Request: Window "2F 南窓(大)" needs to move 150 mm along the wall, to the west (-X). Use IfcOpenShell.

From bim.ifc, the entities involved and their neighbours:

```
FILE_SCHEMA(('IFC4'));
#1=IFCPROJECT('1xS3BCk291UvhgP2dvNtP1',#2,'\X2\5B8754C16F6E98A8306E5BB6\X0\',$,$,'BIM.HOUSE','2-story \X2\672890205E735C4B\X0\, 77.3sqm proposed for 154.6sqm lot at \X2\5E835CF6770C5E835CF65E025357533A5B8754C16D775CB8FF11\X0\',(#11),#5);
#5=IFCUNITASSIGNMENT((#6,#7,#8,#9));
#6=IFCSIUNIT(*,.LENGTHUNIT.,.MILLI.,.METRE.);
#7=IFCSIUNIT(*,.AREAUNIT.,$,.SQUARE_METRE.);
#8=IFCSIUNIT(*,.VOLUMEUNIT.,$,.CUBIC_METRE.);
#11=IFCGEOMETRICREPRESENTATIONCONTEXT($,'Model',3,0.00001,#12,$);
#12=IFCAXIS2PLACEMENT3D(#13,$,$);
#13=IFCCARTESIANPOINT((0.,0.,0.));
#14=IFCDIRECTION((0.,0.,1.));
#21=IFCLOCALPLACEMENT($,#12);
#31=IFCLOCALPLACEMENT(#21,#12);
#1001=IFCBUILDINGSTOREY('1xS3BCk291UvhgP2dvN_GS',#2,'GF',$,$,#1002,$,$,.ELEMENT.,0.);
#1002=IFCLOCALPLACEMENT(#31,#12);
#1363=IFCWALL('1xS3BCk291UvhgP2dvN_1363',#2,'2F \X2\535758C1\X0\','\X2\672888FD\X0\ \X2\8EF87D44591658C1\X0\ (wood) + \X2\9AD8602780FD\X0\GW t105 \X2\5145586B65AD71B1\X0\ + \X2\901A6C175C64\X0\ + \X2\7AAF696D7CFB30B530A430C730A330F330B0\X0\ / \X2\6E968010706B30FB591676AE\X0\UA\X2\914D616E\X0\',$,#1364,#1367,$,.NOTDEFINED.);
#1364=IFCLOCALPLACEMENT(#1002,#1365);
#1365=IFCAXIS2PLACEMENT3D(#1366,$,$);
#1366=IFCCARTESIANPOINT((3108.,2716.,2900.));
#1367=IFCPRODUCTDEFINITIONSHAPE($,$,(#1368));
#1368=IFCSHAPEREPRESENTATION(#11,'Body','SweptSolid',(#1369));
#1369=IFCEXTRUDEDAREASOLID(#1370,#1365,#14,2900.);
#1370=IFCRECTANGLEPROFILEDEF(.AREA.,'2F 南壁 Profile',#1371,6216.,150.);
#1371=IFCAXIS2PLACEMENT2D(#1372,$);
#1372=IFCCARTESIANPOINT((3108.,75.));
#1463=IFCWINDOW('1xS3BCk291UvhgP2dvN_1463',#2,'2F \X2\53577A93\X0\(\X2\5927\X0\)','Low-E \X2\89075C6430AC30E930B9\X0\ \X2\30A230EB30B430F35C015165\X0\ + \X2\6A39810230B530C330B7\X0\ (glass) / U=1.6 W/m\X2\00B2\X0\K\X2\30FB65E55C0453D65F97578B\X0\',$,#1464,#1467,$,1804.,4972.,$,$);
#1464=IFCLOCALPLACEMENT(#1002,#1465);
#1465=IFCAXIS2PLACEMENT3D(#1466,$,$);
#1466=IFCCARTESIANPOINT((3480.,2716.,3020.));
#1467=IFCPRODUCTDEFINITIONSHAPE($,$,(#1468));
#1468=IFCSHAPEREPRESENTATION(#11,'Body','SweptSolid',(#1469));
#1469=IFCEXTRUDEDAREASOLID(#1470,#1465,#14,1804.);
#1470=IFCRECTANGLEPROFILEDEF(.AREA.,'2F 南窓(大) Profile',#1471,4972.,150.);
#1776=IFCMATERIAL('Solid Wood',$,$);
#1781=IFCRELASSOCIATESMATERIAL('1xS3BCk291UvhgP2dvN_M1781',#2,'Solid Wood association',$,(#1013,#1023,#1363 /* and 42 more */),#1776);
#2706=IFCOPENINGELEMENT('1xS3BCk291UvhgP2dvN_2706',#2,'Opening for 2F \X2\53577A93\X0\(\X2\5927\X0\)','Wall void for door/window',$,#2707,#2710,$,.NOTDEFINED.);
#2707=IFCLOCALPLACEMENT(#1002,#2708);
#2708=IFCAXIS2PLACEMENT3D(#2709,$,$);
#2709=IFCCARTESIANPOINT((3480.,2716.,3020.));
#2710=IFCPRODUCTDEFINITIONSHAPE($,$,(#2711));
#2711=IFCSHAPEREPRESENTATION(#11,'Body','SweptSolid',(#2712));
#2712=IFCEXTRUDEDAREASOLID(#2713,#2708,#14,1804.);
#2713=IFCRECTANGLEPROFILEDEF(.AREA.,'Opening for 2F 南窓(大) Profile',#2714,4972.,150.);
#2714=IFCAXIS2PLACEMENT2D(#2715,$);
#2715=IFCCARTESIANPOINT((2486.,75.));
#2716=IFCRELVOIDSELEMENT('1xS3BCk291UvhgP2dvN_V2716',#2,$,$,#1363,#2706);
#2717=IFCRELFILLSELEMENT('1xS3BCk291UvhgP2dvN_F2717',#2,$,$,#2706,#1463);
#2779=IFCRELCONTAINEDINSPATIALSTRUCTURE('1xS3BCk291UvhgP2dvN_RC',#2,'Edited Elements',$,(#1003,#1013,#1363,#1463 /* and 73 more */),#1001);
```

```python
import ifcopenshell
import ifcopenshell.api.geometry
import ifcopenshell.util.placement
import ifcopenshell.util.unit

model = ifcopenshell.open("bim.ifc")
unit_scale = ifcopenshell.util.unit.calculate_unit_scale(model)

window = model.by_guid("1xS3BCk291UvhgP2dvN_1463")
opening = window.FillsVoids[0].RelatingOpeningElement
wall = opening.VoidsElements[0].RelatingBuildingElement

wall_matrix = ifcopenshell.util.placement.get_local_placement(wall.ObjectPlacement)
shift = wall_matrix[:3, 0] * -0.15 / unit_scale
before = ifcopenshell.util.placement.get_local_placement(window.ObjectPlacement)[:3, 3].copy()

# The window is not placed relative to its opening, so move both.
for product in (opening, window):
    matrix = ifcopenshell.util.placement.get_local_placement(product.ObjectPlacement)
    matrix[:3, 3] += shift
    ifcopenshell.api.geometry.edit_object_placement(model, product=product, matrix=matrix, is_si=False)

after = ifcopenshell.util.placement.get_local_placement(window.ObjectPlacement)[:3, 3]
print("window moved by", (after - before).round(3) + 0.0)

model.write("bim_v2.ifc")
```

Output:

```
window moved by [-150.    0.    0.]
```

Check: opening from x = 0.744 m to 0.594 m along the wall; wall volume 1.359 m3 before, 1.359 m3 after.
